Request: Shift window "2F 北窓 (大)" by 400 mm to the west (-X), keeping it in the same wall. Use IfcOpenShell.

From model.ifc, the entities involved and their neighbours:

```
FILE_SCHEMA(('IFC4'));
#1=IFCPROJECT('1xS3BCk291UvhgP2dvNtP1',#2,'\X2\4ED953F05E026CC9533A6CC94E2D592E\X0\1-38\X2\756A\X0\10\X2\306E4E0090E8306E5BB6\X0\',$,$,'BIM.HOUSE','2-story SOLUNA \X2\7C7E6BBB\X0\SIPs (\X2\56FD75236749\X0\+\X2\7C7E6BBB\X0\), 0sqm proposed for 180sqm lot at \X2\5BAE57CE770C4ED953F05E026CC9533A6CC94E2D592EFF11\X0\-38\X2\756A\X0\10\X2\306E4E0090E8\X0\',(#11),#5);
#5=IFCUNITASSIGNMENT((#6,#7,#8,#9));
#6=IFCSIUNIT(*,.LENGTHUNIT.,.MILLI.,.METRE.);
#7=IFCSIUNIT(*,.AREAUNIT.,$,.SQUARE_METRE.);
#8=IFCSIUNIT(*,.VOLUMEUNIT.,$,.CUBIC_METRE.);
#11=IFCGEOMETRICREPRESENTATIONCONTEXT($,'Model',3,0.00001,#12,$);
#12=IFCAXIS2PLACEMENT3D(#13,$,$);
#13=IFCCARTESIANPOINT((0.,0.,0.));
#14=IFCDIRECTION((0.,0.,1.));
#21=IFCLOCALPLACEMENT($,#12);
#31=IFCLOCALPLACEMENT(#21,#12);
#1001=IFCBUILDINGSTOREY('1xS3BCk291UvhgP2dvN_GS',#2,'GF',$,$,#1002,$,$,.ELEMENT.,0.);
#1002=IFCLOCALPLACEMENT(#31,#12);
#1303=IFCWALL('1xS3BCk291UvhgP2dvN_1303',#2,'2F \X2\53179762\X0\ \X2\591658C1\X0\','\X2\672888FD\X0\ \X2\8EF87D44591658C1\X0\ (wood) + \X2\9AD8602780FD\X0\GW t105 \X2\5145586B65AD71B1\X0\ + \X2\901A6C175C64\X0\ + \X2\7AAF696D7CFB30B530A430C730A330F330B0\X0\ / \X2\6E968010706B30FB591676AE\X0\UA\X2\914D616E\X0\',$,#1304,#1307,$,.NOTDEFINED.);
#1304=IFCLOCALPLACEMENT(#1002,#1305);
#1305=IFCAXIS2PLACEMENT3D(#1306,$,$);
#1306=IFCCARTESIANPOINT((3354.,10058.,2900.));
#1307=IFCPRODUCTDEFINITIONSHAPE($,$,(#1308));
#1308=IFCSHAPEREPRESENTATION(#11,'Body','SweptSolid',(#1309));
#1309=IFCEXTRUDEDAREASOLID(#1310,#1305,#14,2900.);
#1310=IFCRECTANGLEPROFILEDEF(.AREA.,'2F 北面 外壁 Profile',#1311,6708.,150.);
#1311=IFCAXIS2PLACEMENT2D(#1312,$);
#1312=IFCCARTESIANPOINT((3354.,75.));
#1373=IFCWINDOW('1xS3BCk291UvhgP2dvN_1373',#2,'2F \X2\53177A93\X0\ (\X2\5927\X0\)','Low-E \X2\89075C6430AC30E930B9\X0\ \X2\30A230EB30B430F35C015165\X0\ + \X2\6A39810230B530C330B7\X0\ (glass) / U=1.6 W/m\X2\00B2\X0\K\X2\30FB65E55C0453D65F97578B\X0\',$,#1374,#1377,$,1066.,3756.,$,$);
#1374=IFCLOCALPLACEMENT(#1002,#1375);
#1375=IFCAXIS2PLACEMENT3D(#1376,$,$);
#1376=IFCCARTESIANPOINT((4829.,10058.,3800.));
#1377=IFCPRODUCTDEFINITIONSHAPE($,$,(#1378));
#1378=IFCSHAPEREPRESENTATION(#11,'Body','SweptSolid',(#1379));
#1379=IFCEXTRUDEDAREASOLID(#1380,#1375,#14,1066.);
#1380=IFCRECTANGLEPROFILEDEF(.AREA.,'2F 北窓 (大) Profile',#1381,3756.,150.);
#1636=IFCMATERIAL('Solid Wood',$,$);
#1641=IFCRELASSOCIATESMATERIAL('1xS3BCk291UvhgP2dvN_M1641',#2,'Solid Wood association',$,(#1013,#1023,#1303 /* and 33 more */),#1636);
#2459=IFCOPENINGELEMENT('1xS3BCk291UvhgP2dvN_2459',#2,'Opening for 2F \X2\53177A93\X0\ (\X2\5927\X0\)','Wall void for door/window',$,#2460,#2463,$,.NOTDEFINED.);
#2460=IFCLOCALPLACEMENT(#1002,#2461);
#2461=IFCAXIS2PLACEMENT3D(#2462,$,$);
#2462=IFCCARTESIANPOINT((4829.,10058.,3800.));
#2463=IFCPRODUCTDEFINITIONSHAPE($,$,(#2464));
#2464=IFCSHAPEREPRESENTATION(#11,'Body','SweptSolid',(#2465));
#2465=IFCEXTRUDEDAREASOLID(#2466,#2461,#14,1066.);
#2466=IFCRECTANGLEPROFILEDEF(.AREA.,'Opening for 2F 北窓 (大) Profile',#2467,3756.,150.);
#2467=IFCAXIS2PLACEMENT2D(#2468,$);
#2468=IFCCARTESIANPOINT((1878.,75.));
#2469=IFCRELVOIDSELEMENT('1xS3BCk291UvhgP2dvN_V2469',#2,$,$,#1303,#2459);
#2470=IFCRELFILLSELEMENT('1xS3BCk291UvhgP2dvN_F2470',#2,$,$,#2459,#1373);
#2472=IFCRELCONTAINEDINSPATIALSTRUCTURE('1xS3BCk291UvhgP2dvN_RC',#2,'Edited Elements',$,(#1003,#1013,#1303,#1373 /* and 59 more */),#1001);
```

```python
import ifcopenshell
import ifcopenshell.api.geometry
import ifcopenshell.util.placement

model = ifcopenshell.open("model.ifc")

window = model.by_guid("1xS3BCk291UvhgP2dvN_1373")
opening = window.FillsVoids[0].RelatingOpeningElement
wall = opening.VoidsElements[0].RelatingBuildingElement

wall_matrix = ifcopenshell.util.placement.get_local_placement(wall.ObjectPlacement)
shift = wall_matrix[:3, 0] * -400.0
before = ifcopenshell.util.placement.get_local_placement(window.ObjectPlacement)[:3, 3].copy()

# The window is not placed relative to its opening, so move both.
for product in (opening, window):
    matrix = ifcopenshell.util.placement.get_local_placement(product.ObjectPlacement)
    matrix[:3, 3] += shift
    ifcopenshell.api.geometry.edit_object_placement(model, product=product, matrix=matrix, is_si=False)

after = ifcopenshell.util.placement.get_local_placement(window.ObjectPlacement)[:3, 3]
print("window moved by", (after - before).round(3) + 0.0)

model.write("model_v2.ifc")
```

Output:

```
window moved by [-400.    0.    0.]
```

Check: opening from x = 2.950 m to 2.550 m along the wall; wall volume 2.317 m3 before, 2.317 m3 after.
